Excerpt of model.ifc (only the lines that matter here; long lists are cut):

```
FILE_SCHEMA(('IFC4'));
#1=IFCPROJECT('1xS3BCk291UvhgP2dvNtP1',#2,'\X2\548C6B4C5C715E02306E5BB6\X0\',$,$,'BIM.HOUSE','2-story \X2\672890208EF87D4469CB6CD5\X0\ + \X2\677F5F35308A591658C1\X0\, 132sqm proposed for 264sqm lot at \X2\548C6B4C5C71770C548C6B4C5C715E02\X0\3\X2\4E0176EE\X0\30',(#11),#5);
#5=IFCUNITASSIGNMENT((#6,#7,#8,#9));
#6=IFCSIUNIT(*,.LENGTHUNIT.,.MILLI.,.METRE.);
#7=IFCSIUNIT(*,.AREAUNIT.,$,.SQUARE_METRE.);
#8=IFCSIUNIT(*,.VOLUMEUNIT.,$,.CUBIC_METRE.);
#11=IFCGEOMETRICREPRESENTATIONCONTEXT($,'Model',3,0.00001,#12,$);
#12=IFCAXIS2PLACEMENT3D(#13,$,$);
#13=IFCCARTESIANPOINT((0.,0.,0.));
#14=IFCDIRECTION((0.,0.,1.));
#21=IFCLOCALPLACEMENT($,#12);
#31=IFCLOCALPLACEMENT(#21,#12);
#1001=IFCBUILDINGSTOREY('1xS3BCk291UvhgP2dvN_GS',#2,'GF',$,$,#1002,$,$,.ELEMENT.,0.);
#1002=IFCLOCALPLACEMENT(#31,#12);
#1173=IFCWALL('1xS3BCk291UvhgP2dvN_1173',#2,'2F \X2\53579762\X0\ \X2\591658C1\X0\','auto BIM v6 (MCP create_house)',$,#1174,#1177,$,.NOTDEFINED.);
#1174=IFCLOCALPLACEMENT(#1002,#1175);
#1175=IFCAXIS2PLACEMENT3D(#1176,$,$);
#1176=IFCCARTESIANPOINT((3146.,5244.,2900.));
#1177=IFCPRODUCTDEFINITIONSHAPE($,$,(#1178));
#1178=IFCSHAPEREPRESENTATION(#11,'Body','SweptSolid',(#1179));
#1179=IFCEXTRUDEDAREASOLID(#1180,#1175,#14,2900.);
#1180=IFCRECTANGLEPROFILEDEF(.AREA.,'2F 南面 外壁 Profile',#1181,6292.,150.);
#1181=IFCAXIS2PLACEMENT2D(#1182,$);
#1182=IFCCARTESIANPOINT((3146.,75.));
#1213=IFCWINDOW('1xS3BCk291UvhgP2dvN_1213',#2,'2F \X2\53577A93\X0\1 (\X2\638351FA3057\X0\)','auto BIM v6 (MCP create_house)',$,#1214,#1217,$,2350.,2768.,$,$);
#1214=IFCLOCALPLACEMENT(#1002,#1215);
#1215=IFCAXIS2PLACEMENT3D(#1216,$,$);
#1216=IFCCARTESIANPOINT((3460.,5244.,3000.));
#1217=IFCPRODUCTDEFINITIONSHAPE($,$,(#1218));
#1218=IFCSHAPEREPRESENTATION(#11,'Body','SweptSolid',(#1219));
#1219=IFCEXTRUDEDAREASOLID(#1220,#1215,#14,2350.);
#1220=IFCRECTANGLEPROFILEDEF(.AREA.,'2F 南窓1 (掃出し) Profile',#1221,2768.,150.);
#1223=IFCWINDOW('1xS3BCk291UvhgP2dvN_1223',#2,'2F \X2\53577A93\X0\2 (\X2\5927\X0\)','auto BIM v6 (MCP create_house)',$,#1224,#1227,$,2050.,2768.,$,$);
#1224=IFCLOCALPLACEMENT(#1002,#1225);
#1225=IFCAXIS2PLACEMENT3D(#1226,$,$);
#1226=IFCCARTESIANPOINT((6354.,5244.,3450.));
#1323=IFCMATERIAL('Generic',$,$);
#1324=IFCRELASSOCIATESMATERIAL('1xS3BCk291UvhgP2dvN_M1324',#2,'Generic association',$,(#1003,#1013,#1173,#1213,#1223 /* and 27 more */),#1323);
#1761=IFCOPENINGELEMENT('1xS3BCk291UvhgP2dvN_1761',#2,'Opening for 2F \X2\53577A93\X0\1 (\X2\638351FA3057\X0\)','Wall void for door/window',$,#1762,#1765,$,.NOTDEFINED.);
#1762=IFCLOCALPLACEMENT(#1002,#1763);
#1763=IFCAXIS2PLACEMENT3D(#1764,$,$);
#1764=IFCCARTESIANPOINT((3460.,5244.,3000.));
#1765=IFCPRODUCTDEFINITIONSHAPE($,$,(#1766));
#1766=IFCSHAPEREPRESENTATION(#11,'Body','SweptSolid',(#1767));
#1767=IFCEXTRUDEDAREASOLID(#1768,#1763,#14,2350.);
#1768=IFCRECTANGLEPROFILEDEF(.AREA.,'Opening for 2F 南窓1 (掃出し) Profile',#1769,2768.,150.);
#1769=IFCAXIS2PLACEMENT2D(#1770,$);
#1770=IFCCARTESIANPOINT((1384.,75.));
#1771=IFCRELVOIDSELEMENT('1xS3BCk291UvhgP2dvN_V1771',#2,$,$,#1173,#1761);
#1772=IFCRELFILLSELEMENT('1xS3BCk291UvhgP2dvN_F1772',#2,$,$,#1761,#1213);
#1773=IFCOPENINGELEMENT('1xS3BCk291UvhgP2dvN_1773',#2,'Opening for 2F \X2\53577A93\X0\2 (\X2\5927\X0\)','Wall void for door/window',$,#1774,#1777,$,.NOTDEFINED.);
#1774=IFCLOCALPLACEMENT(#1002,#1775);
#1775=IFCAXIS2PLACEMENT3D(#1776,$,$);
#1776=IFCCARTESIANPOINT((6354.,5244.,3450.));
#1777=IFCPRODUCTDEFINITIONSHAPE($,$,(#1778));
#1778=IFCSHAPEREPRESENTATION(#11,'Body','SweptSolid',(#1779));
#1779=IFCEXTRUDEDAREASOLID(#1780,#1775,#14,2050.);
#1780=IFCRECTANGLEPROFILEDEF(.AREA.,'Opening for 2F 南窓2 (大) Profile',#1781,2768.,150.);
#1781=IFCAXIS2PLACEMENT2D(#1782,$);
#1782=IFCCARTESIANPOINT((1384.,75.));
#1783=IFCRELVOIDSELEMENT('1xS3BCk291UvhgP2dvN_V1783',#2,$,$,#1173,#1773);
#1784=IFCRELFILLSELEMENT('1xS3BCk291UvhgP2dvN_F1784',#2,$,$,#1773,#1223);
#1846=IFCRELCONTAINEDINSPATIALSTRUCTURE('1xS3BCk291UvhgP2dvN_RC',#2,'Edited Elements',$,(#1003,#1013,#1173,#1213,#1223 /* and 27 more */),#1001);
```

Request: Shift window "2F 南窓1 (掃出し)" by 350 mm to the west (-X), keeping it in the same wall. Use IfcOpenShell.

```python
import ifcopenshell
import ifcopenshell.api.geometry
import ifcopenshell.util.placement
import ifcopenshell.util.unit

model = ifcopenshell.open("model.ifc")
unit_scale = ifcopenshell.util.unit.calculate_unit_scale(model)

window = model.by_id(1213)
opening = window.FillsVoids[0].RelatingOpeningElement
wall = opening.VoidsElements[0].RelatingBuildingElement

wall_matrix = ifcopenshell.util.placement.get_local_placement(wall.ObjectPlacement)
shift = wall_matrix[:3, 0] * -0.35 / unit_scale
before = ifcopenshell.util.placement.get_local_placement(window.ObjectPlacement)[:3, 3].copy()

# The window is not placed relative to its opening, so move both.
for product in (opening, window):
    matrix = ifcopenshell.util.placement.get_local_placement(product.ObjectPlacement)
    matrix[:3, 3] += shift
    ifcopenshell.api.geometry.edit_object_placement(model, product=product, matrix=matrix, is_si=False)

after = ifcopenshell.util.placement.get_local_placement(window.ObjectPlacement)[:3, 3]
print("window moved by", (after - before).round(3) + 0.0)

model.write("model_rev.ifc")
```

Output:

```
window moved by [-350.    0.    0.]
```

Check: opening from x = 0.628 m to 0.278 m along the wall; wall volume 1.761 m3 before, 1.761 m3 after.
